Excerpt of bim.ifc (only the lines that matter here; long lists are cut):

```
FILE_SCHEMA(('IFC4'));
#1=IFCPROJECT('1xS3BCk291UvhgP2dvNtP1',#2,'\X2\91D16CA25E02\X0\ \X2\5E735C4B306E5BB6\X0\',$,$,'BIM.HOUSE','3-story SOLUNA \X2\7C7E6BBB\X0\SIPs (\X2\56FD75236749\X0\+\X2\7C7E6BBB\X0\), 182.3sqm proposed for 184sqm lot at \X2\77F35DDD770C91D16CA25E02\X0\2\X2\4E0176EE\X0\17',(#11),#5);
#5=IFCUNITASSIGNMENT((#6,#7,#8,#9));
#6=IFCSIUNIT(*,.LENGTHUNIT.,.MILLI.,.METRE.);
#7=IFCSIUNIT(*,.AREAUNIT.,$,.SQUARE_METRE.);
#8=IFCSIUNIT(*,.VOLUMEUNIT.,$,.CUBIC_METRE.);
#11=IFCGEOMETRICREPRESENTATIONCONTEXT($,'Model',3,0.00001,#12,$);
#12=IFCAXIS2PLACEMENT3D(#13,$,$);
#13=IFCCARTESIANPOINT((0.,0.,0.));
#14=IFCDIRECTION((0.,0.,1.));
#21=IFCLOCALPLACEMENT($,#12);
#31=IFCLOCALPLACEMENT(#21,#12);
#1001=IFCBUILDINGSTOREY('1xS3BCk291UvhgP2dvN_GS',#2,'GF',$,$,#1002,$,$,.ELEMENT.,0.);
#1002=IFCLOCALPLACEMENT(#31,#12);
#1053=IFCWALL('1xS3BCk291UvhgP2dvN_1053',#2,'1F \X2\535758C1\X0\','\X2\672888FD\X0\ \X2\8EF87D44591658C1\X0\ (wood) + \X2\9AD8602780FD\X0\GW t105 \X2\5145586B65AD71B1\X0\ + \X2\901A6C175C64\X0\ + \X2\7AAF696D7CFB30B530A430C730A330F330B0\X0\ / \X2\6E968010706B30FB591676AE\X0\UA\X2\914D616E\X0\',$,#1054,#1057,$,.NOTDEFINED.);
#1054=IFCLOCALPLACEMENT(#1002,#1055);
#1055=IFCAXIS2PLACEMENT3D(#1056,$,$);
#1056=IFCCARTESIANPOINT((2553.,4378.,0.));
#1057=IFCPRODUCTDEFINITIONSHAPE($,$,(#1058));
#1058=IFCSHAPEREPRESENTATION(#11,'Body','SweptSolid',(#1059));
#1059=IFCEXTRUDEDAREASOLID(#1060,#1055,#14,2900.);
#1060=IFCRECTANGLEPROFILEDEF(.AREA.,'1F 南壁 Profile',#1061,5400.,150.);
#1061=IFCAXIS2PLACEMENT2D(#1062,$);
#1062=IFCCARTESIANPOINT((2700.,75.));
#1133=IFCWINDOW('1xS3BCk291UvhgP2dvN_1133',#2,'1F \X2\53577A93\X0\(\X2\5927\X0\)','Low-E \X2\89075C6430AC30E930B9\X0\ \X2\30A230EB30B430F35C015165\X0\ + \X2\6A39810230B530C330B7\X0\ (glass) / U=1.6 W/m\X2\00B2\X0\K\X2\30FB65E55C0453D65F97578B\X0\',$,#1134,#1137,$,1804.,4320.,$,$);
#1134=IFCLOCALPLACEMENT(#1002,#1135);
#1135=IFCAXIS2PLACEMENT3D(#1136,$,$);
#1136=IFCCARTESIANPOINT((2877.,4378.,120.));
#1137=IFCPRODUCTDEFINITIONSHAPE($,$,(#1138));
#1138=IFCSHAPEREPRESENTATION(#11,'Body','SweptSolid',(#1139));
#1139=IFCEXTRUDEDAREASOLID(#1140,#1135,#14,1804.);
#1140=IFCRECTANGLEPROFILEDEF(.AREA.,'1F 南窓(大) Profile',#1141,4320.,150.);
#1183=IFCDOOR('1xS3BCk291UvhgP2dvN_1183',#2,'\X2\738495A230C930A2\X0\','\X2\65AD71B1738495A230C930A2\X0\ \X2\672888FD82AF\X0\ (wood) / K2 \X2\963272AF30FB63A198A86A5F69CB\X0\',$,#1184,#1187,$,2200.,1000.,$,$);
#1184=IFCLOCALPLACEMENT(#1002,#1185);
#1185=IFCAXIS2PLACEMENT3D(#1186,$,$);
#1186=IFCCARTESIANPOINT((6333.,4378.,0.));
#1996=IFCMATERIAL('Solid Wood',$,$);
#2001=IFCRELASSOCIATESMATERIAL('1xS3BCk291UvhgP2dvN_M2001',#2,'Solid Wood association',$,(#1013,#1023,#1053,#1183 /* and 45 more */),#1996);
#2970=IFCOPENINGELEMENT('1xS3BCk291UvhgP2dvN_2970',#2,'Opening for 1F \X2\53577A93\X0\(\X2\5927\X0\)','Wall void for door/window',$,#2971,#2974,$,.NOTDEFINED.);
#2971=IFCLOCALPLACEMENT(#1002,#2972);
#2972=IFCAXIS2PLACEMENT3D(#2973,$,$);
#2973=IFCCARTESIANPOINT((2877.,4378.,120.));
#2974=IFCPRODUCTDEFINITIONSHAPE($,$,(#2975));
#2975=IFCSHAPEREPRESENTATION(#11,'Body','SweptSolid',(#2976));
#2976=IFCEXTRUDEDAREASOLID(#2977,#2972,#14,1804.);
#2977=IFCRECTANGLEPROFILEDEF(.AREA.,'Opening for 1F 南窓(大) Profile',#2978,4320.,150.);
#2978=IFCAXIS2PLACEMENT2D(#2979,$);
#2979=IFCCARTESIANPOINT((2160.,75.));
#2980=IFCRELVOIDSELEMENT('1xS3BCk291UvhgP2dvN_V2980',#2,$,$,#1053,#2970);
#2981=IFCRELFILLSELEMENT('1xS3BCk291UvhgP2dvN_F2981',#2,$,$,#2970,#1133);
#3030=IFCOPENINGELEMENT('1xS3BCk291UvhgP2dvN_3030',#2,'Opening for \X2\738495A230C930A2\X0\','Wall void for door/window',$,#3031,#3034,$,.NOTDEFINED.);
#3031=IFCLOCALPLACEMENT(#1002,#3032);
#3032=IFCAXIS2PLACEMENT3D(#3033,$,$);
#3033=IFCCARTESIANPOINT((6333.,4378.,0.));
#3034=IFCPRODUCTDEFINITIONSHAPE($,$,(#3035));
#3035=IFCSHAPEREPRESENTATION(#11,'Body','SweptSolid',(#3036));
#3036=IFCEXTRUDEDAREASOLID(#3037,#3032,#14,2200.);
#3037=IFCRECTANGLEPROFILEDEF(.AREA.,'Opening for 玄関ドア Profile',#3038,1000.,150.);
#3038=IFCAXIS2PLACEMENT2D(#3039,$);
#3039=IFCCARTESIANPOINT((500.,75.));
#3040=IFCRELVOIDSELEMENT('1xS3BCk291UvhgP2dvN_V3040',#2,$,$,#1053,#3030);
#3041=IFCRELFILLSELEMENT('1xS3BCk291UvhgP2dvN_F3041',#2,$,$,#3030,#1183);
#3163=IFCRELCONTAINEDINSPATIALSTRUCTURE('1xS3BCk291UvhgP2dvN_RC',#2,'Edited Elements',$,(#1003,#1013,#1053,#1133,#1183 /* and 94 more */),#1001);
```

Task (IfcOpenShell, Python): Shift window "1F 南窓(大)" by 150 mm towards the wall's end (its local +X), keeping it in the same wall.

```python
import ifcopenshell
import ifcopenshell.api.geometry
import ifcopenshell.util.placement
import ifcopenshell.util.unit

model = ifcopenshell.open("bim.ifc")
unit_scale = ifcopenshell.util.unit.calculate_unit_scale(model)

window = model.by_id(1133)
opening = window.FillsVoids[0].RelatingOpeningElement
wall = opening.VoidsElements[0].RelatingBuildingElement

wall_matrix = ifcopenshell.util.placement.get_local_placement(wall.ObjectPlacement)
shift = wall_matrix[:3, 0] * 0.15 / unit_scale
before = ifcopenshell.util.placement.get_local_placement(window.ObjectPlacement)[:3, 3].copy()

# The window is not placed relative to its opening, so move both.
for product in (opening, window):
    matrix = ifcopenshell.util.placement.get_local_placement(product.ObjectPlacement)
    matrix[:3, 3] += shift
    ifcopenshell.api.geometry.edit_object_placement(model, product=product, matrix=matrix, is_si=False)

after = ifcopenshell.util.placement.get_local_placement(window.ObjectPlacement)[:3, 3]
print("window moved by", (after - before).round(3) + 0.0)

model.write("bim-out.ifc")
```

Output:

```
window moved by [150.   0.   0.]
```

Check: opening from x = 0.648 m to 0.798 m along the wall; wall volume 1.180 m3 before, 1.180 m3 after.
